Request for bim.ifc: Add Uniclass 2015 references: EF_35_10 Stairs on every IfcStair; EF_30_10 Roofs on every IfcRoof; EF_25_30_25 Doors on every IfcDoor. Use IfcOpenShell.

First a look at what the model holds.

```python
import ifcopenshell

model = ifcopenshell.open("bim.ifc")
print(model.schema)
print("classifications:", [c.Name for c in model.by_type("IfcClassification")])
for ifc_class in ("IfcDoor", "IfcRoof", "IfcStair", "IfcWall", "IfcWindow"):
    print(ifc_class, len(model.by_type(ifc_class)))
```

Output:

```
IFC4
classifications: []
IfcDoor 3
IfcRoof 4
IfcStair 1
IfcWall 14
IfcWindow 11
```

```python
import ifcopenshell
import ifcopenshell.api.classification

model = ifcopenshell.open("bim.ifc")

system = ifcopenshell.api.classification.add_classification(model, classification="Uniclass 2015")

codes = {
    "IfcStair": ("EF_35_10", "Stairs"),
    "IfcRoof": ("EF_30_10", "Roofs"),
    "IfcDoor": ("EF_25_30_25", "Doors"),
}
for ifc_class, (code, name) in codes.items():
    products = model.by_type(ifc_class)
    ifcopenshell.api.classification.add_reference(
        model, products=products, classification=system, identification=code, name=name
    )
    print(code, len(products))

model.write("bim_edited.ifc")
```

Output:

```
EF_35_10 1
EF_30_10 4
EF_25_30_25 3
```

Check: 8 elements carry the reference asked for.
